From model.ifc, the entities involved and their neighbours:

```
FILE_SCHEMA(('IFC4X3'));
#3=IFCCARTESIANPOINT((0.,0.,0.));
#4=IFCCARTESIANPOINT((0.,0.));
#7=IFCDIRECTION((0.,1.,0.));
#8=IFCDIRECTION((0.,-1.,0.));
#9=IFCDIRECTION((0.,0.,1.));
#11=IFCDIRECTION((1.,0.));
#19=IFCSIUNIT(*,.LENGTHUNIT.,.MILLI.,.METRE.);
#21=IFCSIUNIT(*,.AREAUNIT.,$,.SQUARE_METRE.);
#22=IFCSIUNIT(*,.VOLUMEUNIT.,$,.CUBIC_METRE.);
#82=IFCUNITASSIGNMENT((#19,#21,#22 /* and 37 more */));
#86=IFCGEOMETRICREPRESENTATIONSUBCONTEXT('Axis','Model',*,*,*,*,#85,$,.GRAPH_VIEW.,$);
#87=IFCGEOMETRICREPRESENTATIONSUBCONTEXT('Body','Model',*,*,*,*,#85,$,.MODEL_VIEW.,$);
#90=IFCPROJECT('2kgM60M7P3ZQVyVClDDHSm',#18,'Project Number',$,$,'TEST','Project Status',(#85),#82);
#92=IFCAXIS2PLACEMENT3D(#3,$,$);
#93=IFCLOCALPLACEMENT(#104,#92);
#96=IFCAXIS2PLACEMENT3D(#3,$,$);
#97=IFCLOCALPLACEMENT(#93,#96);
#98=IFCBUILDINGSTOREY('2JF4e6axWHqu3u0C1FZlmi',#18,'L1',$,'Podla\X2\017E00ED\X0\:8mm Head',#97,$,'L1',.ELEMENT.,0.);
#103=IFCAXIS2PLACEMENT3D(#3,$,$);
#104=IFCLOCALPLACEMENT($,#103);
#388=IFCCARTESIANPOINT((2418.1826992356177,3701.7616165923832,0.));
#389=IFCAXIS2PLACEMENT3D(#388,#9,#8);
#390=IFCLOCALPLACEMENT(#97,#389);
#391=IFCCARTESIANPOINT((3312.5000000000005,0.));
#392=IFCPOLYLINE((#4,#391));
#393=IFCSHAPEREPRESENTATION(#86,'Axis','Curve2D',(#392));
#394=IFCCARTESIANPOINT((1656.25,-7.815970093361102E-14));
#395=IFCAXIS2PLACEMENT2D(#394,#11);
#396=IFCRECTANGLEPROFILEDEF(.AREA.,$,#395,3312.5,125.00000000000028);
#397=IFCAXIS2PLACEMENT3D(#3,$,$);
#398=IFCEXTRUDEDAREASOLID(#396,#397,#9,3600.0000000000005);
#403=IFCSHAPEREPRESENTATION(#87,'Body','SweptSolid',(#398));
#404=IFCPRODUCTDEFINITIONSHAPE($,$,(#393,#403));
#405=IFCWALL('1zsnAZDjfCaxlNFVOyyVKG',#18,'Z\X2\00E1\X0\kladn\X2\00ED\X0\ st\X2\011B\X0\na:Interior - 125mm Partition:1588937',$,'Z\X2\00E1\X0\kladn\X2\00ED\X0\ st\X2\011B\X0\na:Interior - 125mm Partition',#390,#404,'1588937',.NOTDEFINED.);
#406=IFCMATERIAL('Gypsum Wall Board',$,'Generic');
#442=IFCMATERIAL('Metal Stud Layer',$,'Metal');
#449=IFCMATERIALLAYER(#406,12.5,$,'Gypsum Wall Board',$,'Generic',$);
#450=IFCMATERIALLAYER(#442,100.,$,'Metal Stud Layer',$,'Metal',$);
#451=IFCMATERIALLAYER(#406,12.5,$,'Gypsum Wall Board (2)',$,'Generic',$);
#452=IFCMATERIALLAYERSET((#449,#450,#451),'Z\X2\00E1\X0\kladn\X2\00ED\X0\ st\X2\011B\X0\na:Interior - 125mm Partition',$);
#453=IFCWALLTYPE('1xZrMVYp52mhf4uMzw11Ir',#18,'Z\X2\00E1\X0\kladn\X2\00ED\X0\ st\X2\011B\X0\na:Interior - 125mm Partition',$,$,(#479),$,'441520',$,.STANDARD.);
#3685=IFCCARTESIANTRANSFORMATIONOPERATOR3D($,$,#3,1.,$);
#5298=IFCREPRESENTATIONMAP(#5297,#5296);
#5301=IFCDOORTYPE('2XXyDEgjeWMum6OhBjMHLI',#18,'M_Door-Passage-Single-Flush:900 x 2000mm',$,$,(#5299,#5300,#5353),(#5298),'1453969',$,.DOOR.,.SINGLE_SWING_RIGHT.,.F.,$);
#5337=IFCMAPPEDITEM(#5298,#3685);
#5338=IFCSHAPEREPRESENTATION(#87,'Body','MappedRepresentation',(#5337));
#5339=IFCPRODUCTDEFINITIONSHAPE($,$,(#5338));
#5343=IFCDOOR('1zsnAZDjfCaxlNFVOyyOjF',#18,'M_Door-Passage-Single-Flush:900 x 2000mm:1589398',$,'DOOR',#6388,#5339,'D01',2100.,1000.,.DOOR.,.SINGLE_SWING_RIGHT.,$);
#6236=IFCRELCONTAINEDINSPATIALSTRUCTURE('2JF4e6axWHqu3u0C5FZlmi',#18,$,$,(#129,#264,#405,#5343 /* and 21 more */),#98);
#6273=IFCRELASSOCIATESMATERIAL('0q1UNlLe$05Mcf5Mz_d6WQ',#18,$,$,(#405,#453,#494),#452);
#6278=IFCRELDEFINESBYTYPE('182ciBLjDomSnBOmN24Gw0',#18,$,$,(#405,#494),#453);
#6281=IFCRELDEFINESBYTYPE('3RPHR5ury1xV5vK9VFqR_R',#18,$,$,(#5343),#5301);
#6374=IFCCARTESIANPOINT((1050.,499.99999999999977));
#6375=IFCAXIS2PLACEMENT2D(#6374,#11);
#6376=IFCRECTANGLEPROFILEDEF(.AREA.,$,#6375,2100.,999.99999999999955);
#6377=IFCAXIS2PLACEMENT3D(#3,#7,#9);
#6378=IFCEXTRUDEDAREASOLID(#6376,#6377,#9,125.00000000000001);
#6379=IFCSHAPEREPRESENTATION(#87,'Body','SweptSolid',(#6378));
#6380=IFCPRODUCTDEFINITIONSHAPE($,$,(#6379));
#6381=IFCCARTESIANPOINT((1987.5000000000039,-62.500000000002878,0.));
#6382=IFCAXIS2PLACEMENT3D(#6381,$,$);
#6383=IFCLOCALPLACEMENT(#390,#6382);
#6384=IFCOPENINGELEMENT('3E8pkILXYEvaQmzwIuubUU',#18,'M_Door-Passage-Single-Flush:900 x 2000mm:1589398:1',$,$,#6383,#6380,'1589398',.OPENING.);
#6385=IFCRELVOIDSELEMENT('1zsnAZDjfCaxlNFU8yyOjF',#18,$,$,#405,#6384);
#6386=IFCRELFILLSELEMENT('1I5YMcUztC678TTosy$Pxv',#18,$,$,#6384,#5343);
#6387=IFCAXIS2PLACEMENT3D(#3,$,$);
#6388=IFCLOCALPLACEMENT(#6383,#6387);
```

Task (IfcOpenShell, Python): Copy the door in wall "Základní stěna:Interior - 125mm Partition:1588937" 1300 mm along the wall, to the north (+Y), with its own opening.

```python
import ifcopenshell
import ifcopenshell.api.feature
import ifcopenshell.api.geometry
import ifcopenshell.api.root
import ifcopenshell.geom
import ifcopenshell.util.element
import ifcopenshell.util.placement
import ifcopenshell.util.shape
import ifcopenshell.util.unit

model = ifcopenshell.open("model.ifc")
unit_scale = ifcopenshell.util.unit.calculate_unit_scale(model)
settings = ifcopenshell.geom.settings()


def volume(element):
    """Net volume in cubic metres, openings subtracted."""
    shape = ifcopenshell.geom.create_shape(settings, element)
    return ifcopenshell.util.shape.get_volume(shape.geometry)


def reuse_history(source, copy):
    """copy_class also copies each property set's owner history, people and application; keep the originals."""
    for rel in copy.IsDefinedBy:
        if rel.is_a("IfcRelDefinesByProperties") and (history := rel.RelatingPropertyDefinition.OwnerHistory):
            rel.RelatingPropertyDefinition.OwnerHistory = source.OwnerHistory
            ifcopenshell.util.element.remove_deep2(model, history)


door = model.by_guid("1zsnAZDjfCaxlNFVOyyOjF")
opening = door.FillsVoids[0].RelatingOpeningElement
wall = opening.VoidsElements[0].RelatingBuildingElement
before = volume(wall)
shift = ifcopenshell.util.placement.get_local_placement(wall.ObjectPlacement)[:3, 0] * -1.3 / unit_scale

# copy_class copies the void relationship, type, container and properties, but no geometry.
new_opening = ifcopenshell.api.root.copy_class(model, product=opening)
new_opening.Representation = ifcopenshell.util.element.copy_deep(
    model, opening.Representation, exclude=["IfcGeometricRepresentationContext", "IfcRepresentationMap"]
)
new_opening.Name = "M_Door-Passage-Single-Flush:900 x 2000mm"
new_opening.Tag = None
new_door = ifcopenshell.api.root.copy_class(model, product=door)
new_door.Representation = ifcopenshell.util.element.copy_deep(
    model, door.Representation, exclude=["IfcGeometricRepresentationContext", "IfcRepresentationMap"]
)
new_door.Name = "M_Door-Passage-Single-Flush:900 x 2000mm"
new_door.Tag = None
reuse_history(door, new_door)
ifcopenshell.api.feature.add_filling(model, opening=new_opening, element=new_door)

for old, new in ((opening, new_opening), (door, new_door)):
    matrix = ifcopenshell.util.placement.get_local_placement(old.ObjectPlacement)
    matrix[:3, 3] += shift
    ifcopenshell.api.geometry.edit_object_placement(model, product=new, matrix=matrix, is_si=False)

after = volume(wall)

print(f"wall volume {before:.3f} -> {after:.3f} m3")

model.write("model_edited.ifc")
```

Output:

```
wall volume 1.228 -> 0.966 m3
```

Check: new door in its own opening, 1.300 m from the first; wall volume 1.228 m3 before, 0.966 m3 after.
